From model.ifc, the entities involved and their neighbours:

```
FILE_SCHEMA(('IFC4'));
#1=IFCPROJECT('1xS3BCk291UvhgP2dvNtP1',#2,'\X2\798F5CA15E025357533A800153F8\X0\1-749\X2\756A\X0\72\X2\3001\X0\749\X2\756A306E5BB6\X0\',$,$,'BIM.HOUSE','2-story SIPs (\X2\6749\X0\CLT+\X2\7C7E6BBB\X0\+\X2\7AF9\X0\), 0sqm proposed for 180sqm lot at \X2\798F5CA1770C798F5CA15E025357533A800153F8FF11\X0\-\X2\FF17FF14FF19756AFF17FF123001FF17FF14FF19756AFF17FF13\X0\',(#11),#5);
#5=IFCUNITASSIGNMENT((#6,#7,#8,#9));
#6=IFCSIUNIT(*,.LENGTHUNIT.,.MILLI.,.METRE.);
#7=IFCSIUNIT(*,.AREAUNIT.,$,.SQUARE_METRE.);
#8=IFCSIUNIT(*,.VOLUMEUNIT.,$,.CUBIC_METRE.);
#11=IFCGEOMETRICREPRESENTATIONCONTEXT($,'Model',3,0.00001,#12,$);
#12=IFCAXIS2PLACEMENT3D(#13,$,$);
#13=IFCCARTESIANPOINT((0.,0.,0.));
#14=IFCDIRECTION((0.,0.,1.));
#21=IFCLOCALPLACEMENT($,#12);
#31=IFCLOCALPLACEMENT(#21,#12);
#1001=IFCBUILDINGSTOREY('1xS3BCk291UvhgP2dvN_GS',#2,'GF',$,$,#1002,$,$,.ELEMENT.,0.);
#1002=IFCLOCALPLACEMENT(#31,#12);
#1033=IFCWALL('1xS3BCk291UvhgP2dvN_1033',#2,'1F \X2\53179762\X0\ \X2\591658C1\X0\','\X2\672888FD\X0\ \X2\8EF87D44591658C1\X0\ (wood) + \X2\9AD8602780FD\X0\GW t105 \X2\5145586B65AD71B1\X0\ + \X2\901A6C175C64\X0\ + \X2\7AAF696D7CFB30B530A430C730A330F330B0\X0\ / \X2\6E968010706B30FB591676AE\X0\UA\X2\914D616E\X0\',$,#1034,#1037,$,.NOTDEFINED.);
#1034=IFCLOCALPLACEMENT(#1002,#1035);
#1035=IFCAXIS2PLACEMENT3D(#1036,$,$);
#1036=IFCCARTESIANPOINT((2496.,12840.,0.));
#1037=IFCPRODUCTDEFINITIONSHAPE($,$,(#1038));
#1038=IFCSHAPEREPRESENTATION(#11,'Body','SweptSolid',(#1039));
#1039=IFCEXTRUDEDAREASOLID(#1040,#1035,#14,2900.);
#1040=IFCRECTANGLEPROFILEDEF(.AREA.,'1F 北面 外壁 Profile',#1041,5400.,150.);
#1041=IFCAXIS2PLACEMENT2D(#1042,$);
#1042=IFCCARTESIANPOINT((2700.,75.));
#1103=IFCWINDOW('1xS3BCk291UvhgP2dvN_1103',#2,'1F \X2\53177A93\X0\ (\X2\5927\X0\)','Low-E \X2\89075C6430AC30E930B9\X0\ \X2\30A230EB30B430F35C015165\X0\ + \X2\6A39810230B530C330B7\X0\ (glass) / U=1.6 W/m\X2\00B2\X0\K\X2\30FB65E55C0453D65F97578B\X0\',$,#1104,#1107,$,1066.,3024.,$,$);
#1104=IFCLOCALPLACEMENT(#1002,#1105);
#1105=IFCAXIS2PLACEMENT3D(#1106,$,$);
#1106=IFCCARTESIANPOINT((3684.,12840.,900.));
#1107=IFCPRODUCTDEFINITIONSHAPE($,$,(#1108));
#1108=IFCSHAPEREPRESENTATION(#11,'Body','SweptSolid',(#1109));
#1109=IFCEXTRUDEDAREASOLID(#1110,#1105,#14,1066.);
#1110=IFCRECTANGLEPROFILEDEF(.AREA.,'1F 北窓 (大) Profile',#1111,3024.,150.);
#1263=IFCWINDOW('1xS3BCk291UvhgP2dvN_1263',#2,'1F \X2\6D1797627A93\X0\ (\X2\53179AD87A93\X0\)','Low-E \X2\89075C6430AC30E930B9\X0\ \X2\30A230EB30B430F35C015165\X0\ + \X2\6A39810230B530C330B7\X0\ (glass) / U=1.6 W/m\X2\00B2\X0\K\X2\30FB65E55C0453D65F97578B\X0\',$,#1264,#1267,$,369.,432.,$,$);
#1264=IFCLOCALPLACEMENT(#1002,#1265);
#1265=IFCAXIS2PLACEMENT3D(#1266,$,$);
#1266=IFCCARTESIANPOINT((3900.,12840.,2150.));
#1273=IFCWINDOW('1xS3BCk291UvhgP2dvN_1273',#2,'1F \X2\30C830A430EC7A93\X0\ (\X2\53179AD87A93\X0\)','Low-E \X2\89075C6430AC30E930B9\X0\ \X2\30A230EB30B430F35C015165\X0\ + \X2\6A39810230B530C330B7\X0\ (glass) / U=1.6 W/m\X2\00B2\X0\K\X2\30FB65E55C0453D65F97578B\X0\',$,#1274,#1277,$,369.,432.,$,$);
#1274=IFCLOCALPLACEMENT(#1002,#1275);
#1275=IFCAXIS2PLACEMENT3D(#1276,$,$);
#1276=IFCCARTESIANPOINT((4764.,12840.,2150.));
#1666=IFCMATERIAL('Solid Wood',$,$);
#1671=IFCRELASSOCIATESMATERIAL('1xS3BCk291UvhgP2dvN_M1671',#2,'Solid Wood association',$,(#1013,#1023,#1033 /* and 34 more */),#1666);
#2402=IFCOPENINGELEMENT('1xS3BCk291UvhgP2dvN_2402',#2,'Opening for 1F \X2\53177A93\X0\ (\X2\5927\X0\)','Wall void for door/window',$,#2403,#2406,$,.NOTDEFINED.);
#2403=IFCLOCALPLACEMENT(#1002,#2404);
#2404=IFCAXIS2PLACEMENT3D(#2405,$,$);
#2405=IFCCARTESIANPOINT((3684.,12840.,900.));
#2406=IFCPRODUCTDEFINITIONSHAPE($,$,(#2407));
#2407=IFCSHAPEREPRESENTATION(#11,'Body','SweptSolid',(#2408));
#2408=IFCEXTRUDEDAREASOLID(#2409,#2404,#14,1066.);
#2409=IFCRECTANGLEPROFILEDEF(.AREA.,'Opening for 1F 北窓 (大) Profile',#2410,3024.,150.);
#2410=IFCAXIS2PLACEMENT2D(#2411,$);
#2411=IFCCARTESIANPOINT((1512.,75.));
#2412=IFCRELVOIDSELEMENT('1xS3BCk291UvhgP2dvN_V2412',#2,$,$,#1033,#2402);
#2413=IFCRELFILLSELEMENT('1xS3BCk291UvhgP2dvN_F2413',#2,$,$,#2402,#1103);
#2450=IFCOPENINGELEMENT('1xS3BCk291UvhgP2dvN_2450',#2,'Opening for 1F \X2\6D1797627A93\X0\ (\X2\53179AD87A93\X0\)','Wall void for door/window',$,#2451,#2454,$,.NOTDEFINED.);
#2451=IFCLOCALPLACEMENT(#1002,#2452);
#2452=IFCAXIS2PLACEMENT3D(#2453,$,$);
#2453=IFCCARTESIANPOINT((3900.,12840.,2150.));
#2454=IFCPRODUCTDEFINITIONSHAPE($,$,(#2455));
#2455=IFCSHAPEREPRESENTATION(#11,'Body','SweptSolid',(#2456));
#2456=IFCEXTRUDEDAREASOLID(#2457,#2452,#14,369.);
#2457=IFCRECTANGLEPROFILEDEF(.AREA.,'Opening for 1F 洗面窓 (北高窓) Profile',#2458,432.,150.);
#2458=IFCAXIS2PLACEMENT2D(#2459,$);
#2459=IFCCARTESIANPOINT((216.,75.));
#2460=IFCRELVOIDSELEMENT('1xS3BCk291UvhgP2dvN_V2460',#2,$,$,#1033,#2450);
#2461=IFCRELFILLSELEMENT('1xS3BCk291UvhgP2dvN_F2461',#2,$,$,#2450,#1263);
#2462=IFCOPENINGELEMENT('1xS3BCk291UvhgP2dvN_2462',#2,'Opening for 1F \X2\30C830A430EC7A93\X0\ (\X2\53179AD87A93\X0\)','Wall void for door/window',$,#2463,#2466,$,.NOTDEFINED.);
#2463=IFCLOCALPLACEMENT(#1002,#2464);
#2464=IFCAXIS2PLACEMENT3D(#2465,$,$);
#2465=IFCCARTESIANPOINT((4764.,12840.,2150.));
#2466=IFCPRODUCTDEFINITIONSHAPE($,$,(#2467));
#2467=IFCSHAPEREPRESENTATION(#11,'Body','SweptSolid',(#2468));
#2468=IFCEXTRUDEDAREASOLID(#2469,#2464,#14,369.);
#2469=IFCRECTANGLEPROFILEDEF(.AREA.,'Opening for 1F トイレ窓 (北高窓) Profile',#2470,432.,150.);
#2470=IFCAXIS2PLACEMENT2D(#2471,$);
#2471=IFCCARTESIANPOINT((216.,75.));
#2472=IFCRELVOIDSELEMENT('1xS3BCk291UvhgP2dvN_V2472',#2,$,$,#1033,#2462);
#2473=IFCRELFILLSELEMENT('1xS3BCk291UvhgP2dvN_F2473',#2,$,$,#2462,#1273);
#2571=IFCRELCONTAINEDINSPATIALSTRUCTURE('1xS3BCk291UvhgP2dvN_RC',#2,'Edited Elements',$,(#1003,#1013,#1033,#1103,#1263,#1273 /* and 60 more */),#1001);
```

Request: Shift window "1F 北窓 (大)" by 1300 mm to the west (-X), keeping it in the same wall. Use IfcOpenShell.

```python
import ifcopenshell
import ifcopenshell.api.geometry
import ifcopenshell.util.placement
import ifcopenshell.util.unit

model = ifcopenshell.open("model.ifc")
unit_scale = ifcopenshell.util.unit.calculate_unit_scale(model)

window = model.by_guid("1xS3BCk291UvhgP2dvN_1103")
opening = window.FillsVoids[0].RelatingOpeningElement
wall = opening.VoidsElements[0].RelatingBuildingElement

wall_matrix = ifcopenshell.util.placement.get_local_placement(wall.ObjectPlacement)
shift = wall_matrix[:3, 0] * -1.3 / unit_scale
before = ifcopenshell.util.placement.get_local_placement(window.ObjectPlacement)[:3, 3].copy()

# The window is not placed relative to its opening, so move both.
for product in (opening, window):
    matrix = ifcopenshell.util.placement.get_local_placement(product.ObjectPlacement)
    matrix[:3, 3] += shift
    ifcopenshell.api.geometry.edit_object_placement(model, product=product, matrix=matrix, is_si=False)

after = ifcopenshell.util.placement.get_local_placement(window.ObjectPlacement)[:3, 3]
print("window moved by", (after - before).round(3) + 0.0)

model.write("model_updated.ifc")
```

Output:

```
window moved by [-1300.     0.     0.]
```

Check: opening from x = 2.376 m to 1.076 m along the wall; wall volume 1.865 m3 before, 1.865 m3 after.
